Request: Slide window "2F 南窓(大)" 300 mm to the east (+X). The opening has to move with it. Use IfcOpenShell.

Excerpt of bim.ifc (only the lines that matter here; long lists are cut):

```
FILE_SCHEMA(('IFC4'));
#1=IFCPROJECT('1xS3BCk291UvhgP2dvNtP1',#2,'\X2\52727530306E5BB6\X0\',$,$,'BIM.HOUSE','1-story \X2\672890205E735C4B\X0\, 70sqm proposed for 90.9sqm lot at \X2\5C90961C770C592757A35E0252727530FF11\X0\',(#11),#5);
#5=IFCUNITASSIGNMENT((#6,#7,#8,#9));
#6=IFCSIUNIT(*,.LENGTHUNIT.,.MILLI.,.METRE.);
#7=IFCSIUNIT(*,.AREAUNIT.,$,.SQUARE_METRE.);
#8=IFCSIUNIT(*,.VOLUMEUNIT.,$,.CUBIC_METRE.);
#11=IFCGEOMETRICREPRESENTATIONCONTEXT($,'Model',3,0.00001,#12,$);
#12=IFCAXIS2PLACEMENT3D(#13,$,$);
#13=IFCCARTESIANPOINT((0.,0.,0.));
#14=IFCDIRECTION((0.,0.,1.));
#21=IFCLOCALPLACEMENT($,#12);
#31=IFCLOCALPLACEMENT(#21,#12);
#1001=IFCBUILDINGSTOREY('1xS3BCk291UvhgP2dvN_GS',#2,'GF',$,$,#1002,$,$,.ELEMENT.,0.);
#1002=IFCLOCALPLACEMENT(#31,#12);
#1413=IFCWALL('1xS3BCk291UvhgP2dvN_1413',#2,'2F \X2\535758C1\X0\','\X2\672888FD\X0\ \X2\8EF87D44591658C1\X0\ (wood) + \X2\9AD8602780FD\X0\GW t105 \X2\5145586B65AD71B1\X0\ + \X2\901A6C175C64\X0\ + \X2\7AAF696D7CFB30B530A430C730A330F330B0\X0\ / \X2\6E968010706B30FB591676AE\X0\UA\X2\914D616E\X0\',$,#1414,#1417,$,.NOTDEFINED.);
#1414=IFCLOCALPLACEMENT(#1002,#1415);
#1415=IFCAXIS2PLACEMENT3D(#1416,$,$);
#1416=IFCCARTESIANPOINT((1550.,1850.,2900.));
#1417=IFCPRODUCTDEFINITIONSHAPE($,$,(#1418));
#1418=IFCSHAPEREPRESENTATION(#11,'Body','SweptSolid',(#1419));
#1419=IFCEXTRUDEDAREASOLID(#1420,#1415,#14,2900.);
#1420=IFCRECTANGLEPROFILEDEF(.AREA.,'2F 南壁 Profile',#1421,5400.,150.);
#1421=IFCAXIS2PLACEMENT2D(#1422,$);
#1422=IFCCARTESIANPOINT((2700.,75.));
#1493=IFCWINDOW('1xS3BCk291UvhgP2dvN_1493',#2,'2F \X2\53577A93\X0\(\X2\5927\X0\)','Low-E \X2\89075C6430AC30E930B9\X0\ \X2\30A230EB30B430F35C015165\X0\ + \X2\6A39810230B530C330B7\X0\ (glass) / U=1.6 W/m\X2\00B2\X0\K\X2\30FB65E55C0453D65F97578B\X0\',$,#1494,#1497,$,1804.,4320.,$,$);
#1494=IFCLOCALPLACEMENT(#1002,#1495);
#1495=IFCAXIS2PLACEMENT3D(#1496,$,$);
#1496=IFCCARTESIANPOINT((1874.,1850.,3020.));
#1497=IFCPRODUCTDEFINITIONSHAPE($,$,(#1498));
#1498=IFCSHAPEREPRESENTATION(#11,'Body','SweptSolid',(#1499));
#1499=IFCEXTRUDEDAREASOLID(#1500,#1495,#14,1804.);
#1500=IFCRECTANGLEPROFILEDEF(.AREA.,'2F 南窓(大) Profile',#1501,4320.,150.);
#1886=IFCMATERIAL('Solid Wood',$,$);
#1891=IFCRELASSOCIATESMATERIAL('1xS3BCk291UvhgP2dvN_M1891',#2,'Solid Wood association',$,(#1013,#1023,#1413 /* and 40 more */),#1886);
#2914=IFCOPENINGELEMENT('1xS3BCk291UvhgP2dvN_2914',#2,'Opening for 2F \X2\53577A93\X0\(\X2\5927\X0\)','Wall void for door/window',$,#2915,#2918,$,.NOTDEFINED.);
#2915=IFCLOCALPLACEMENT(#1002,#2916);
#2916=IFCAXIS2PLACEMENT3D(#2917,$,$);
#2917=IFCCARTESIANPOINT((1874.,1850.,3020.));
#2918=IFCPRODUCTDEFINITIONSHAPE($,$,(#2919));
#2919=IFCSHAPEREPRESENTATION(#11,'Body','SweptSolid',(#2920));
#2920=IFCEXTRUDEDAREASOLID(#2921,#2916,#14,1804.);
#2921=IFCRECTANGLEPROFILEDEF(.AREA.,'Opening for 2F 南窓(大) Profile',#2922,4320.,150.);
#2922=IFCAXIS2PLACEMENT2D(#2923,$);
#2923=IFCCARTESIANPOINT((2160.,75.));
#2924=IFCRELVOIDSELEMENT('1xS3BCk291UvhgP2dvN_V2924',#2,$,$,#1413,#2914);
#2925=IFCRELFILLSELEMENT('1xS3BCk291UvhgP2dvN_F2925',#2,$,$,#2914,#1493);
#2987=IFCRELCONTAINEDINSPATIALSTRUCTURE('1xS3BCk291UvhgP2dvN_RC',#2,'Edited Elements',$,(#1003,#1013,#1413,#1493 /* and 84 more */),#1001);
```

```python
import ifcopenshell
import ifcopenshell.api.geometry
import ifcopenshell.util.placement

model = ifcopenshell.open("bim.ifc")

window = model.by_guid("1xS3BCk291UvhgP2dvN_1493")
opening = window.FillsVoids[0].RelatingOpeningElement
wall = opening.VoidsElements[0].RelatingBuildingElement

wall_matrix = ifcopenshell.util.placement.get_local_placement(wall.ObjectPlacement)
shift = wall_matrix[:3, 0] * 300.0
before = ifcopenshell.util.placement.get_local_placement(window.ObjectPlacement)[:3, 3].copy()

# The window is not placed relative to its opening, so move both.
for product in (opening, window):
    matrix = ifcopenshell.util.placement.get_local_placement(product.ObjectPlacement)
    matrix[:3, 3] += shift
    ifcopenshell.api.geometry.edit_object_placement(model, product=product, matrix=matrix, is_si=False)

after = ifcopenshell.util.placement.get_local_placement(window.ObjectPlacement)[:3, 3]
print("window moved by", (after - before).round(3) + 0.0)

model.write("bim_updated.ifc")
```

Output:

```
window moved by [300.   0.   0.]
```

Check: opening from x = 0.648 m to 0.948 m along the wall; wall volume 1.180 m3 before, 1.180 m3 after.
